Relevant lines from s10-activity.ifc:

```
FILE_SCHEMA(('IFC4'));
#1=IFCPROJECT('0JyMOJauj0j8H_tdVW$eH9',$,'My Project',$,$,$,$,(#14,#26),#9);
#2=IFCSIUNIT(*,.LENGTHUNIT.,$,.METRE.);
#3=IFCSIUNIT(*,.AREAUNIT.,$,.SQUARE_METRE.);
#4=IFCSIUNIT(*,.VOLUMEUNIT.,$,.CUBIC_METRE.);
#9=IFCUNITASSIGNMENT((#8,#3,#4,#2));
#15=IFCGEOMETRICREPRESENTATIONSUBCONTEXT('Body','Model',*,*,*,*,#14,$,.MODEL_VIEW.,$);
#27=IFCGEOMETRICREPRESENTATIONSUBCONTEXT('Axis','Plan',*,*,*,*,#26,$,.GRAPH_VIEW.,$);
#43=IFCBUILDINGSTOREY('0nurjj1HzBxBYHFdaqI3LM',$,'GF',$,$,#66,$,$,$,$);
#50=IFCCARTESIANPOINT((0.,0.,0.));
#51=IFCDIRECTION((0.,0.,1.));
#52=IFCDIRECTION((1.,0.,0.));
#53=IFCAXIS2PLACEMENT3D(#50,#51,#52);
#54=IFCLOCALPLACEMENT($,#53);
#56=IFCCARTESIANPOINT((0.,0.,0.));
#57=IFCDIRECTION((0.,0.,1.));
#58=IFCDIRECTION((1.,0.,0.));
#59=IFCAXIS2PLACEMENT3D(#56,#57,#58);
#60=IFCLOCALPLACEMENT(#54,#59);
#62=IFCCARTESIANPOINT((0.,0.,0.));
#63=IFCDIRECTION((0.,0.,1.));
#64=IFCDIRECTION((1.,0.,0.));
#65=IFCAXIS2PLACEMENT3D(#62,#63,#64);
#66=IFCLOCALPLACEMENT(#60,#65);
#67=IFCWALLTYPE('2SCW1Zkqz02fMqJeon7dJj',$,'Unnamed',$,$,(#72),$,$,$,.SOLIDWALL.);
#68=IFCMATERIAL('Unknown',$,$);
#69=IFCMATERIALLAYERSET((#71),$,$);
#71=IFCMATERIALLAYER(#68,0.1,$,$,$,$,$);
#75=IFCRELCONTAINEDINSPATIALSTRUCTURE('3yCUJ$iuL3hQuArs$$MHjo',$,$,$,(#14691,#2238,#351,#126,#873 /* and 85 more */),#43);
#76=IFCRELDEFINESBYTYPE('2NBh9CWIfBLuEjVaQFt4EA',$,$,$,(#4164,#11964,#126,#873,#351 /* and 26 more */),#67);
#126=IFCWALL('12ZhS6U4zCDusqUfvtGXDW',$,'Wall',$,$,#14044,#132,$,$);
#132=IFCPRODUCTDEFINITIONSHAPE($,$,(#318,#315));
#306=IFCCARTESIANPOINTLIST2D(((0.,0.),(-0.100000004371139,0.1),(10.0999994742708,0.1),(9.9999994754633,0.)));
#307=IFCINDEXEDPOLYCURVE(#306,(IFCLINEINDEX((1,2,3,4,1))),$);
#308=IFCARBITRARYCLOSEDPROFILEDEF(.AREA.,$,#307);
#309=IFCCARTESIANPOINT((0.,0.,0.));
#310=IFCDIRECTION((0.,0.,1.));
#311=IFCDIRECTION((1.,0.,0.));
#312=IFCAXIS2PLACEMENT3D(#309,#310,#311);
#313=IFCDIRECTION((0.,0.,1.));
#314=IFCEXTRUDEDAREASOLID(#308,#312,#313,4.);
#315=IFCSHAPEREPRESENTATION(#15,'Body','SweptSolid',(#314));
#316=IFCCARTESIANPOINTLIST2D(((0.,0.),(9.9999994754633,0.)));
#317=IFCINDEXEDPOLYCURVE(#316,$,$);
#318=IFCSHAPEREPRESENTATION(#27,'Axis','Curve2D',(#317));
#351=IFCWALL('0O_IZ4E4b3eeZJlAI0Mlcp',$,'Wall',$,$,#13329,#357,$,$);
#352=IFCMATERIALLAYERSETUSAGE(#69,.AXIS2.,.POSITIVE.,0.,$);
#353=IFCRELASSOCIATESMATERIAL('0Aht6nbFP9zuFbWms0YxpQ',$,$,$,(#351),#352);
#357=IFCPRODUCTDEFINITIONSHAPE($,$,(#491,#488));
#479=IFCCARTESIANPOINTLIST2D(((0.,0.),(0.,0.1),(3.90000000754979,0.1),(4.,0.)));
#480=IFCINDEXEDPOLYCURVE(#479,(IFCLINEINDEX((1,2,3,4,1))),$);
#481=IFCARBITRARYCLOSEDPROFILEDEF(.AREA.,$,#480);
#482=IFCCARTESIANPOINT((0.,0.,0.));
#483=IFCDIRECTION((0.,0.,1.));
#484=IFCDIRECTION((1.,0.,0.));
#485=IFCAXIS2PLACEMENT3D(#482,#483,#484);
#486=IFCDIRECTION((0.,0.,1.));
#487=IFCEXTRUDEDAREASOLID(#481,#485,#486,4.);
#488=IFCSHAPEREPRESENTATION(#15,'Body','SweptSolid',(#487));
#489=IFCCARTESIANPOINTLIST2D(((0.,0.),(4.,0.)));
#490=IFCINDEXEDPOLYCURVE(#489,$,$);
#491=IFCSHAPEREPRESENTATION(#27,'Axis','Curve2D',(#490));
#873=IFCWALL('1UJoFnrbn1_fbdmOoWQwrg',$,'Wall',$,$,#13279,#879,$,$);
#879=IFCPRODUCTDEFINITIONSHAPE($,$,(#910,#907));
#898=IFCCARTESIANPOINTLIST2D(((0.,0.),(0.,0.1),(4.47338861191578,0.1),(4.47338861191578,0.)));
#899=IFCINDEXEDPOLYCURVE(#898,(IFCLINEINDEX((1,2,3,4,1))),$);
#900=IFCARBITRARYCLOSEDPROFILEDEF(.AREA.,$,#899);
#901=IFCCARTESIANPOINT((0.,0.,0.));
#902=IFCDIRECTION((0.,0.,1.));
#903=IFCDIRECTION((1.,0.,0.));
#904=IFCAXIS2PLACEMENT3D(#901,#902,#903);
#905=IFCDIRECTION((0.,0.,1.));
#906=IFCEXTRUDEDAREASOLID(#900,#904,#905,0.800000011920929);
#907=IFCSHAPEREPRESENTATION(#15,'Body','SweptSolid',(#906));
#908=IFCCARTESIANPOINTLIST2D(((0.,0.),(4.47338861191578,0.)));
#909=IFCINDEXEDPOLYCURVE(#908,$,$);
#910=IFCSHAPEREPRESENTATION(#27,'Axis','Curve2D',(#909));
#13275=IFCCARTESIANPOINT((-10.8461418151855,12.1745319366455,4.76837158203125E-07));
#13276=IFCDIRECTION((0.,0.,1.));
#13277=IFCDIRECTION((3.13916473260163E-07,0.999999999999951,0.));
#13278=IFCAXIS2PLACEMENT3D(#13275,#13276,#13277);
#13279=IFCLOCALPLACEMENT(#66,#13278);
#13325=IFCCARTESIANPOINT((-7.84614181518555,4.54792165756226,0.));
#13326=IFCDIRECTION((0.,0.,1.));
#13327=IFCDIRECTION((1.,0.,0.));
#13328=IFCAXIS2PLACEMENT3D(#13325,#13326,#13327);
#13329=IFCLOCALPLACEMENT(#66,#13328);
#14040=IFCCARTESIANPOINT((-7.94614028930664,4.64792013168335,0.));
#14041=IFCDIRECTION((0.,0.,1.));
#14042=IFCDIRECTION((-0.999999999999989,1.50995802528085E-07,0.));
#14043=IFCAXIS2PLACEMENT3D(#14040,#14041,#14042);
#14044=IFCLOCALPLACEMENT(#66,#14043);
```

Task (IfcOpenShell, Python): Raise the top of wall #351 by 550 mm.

```python
import ifcopenshell
import ifcopenshell.geom
import ifcopenshell.util.representation
import ifcopenshell.util.shape
import ifcopenshell.util.unit

model = ifcopenshell.open("s10-activity.ifc")
unit_scale = ifcopenshell.util.unit.calculate_unit_scale(model)
settings = ifcopenshell.geom.settings()


def volume(element):
    """Net volume in cubic metres, openings subtracted."""
    shape = ifcopenshell.geom.create_shape(settings, element)
    return ifcopenshell.util.shape.get_volume(shape.geometry)


wall = model.by_guid("0O_IZ4E4b3eeZJlAI0Mlcp")
before = volume(wall)

body = ifcopenshell.util.representation.get_representation(wall, "Model", "Body")
solid = body.Items[0]
old_height = solid.Depth
solid.Depth += 0.55 / unit_scale
after = volume(wall)

print(f"height {old_height:g} -> {solid.Depth:g}, volume {before:.3f} -> {after:.3f} m3")

model.write("s10-activity_edited.ifc")
```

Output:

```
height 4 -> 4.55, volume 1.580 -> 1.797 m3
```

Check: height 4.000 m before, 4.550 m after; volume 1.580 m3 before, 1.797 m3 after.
